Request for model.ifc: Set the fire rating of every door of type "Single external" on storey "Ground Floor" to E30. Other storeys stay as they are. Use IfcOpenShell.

First a look at what the model holds.

```python
import ifcopenshell
import ifcopenshell.util.element

model = ifcopenshell.open("model.ifc")
print(model.schema)
storey = next(s for s in model.by_type("IfcBuildingStorey") if s.Name == "Ground Floor")
doors = [e for e in ifcopenshell.util.element.get_decomposition(storey) if e.is_a("IfcDoor")]
seen = {}
for e in doors:
    element_type = ifcopenshell.util.element.get_type(e)
    key = (element_type.Name if element_type != e and element_type else None, ifcopenshell.util.element.get_pset(e, "Pset_DoorCommon", "FireRating"))
    seen[key] = seen.get(key, 0) + 1
for (name, value), count in sorted(seen.items(), key=str):
    print(count, "x", name, "|", value)
```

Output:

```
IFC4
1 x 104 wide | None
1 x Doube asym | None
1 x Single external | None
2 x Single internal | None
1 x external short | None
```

```python
import ifcopenshell
import ifcopenshell.api.pset
import ifcopenshell.util.element

model = ifcopenshell.open("model.ifc")

storey = next(s for s in model.by_type("IfcBuildingStorey") if s.Name == "Ground Floor")
doors = [e for e in ifcopenshell.util.element.get_decomposition(storey) if e.is_a("IfcDoor")]

count = 0
for e in doors:
    element_type = ifcopenshell.util.element.get_type(e)
    if element_type in (None, e) or element_type.Name != "Single external":
        continue
    # add_pset returns the element's existing set when there is one.
    pset = ifcopenshell.api.pset.add_pset(model, product=e, name="Pset_DoorCommon")
    ifcopenshell.api.pset.edit_pset(model, pset=pset, properties={"FireRating": "E30"})
    count += 1

print(count, "doors updated")

model.write("model-out.ifc")
```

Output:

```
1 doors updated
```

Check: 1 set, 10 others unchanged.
